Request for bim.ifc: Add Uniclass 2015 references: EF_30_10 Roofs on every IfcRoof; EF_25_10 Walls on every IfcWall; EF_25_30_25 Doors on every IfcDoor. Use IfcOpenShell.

First a look at what the model holds.

```python
import ifcopenshell

model = ifcopenshell.open("bim.ifc")
print(model.schema)
print("classifications:", [c.Name for c in model.by_type("IfcClassification")])
for ifc_class in ("IfcDoor", "IfcRoof", "IfcStair", "IfcWall", "IfcWindow"):
    print(ifc_class, len(model.by_type(ifc_class)))
```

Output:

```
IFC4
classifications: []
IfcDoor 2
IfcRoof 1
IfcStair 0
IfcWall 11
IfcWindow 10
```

```python
import ifcopenshell
import ifcopenshell.api.classification

model = ifcopenshell.open("bim.ifc")

system = ifcopenshell.api.classification.add_classification(model, classification="Uniclass 2015")

codes = {
    "IfcRoof": ("EF_30_10", "Roofs"),
    "IfcWall": ("EF_25_10", "Walls"),
    "IfcDoor": ("EF_25_30_25", "Doors"),
}
for ifc_class, (code, name) in codes.items():
    products = model.by_type(ifc_class)
    ifcopenshell.api.classification.add_reference(
        model, products=products, classification=system, identification=code, name=name
    )
    print(code, len(products))

model.write("bim_v2.ifc")
```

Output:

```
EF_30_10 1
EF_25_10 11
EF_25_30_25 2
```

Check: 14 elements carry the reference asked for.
